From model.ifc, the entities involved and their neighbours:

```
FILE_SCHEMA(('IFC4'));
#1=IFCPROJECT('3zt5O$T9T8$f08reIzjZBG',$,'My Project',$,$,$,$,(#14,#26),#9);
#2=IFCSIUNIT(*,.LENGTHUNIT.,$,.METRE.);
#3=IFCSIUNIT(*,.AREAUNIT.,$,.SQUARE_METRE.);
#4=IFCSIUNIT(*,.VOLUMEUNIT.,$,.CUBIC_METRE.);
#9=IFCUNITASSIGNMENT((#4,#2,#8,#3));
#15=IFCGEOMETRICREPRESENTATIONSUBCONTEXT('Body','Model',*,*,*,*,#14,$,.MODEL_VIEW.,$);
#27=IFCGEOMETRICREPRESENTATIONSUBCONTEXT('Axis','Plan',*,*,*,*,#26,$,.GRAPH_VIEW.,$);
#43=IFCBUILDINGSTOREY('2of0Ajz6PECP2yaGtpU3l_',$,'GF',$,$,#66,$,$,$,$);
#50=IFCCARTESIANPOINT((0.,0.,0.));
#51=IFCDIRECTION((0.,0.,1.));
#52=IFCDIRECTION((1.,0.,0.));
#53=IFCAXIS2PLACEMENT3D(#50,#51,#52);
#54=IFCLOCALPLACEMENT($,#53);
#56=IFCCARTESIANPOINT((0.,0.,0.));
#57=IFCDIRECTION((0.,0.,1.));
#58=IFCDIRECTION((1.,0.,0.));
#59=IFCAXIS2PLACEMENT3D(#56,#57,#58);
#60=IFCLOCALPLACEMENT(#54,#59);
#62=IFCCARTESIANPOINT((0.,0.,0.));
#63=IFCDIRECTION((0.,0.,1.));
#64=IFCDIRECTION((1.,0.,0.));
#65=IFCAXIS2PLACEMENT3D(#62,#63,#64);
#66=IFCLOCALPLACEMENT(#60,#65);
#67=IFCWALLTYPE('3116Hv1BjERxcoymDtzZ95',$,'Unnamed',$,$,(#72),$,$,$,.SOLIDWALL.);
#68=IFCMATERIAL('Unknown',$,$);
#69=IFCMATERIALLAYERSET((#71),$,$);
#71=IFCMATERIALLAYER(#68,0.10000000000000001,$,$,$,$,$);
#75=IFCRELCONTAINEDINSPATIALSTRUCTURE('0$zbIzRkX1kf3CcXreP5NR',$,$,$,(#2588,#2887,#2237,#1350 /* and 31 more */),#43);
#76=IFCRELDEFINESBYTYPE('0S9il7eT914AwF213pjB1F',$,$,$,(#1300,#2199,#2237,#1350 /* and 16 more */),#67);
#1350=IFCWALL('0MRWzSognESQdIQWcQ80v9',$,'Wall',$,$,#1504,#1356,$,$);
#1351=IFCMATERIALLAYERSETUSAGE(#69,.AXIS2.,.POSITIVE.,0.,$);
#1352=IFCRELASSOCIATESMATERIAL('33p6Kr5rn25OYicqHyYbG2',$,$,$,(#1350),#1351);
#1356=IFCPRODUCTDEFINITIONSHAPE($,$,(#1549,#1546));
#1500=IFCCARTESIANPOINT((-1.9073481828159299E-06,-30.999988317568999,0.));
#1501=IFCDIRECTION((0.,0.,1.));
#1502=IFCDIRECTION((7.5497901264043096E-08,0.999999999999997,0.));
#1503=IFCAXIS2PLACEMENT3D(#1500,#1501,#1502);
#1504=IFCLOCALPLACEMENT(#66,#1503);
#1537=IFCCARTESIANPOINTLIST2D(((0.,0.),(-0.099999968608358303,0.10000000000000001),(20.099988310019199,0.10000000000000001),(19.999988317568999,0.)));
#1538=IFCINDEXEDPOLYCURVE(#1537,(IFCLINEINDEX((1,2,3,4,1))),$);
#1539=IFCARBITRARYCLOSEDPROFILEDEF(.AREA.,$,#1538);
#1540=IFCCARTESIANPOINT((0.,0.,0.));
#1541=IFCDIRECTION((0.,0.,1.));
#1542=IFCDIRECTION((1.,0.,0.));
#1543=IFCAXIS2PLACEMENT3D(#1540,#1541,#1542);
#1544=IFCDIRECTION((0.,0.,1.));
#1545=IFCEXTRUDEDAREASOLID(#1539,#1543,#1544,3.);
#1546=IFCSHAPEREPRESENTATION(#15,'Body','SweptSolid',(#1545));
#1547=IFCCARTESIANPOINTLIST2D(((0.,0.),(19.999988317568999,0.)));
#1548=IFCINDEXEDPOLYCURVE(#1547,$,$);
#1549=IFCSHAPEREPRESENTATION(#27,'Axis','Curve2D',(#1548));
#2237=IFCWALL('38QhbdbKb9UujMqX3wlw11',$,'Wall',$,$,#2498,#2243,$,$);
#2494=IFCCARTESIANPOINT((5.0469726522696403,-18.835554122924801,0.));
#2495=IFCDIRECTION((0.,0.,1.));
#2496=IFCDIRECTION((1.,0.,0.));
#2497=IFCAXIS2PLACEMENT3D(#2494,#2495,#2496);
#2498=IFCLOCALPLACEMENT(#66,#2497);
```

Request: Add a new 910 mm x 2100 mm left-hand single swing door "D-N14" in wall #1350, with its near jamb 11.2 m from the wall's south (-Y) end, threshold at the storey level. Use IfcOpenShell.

```python
import numpy as np
import ifcopenshell
import ifcopenshell.api.feature
import ifcopenshell.api.geometry
import ifcopenshell.api.root
import ifcopenshell.api.spatial
import ifcopenshell.geom
import ifcopenshell.util.element
import ifcopenshell.util.placement
import ifcopenshell.util.representation
import ifcopenshell.util.shape
import ifcopenshell.util.unit

model = ifcopenshell.open("model.ifc")
unit_scale = ifcopenshell.util.unit.calculate_unit_scale(model)
settings = ifcopenshell.geom.settings()


def volume(element):
    """Net volume in cubic metres, openings subtracted."""
    shape = ifcopenshell.geom.create_shape(settings, element)
    return ifcopenshell.util.shape.get_volume(shape.geometry)


wall = model.by_guid("0MRWzSognESQdIQWcQ80v9")
storey = ifcopenshell.util.element.get_container(wall, ifc_class="IfcBuildingStorey")
context = ifcopenshell.util.representation.get_context(model, "Model", "Body", "MODEL_VIEW")
before = volume(wall)

width, height, from_end, sill = 0.91, 2.1, 11.2, 0.0  # metres

# The wall runs along its own X axis, and the end named is its -X end.
wall_shape = ifcopenshell.geom.create_shape(settings, wall)
x, y, z = ifcopenshell.util.shape.get_vertices(wall_shape.geometry).T
start = x.min() + from_end
face, thickness = float(y.min()), float(y.max() - y.min())
wall_matrix = ifcopenshell.util.placement.get_local_placement(wall.ObjectPlacement)
level = ifcopenshell.util.placement.get_local_placement(storey.ObjectPlacement)[2, 3]


def in_wall(x, y):
    """Placement at x, y metres in the wall's axes, at sill height."""
    matrix = wall_matrix.copy()
    matrix[:, 3] = wall_matrix @ np.array([x / unit_scale, y / unit_scale, 0.0, 1.0])
    matrix[2, 3] = level + sill / unit_scale
    return matrix


# Opening: a box that overshoots both wall faces by 50 mm.
opening = ifcopenshell.api.root.create_entity(model, ifc_class="IfcOpeningElement", predefined_type="OPENING")
box = ifcopenshell.api.geometry.add_wall_representation(
    model, context=context, length=width, height=height, thickness=thickness + 0.1
)
ifcopenshell.api.geometry.assign_representation(model, product=opening, representation=box)
ifcopenshell.api.geometry.edit_object_placement(model, product=opening, matrix=in_wall(start, face - 0.05), is_si=False)
ifcopenshell.api.feature.add_feature(model, feature=opening, element=wall)

door = ifcopenshell.api.root.create_entity(model, ifc_class="IfcDoor", name="D-N14", predefined_type="DOOR")
door.OverallWidth, door.OverallHeight = width / unit_scale, height / unit_scale
door.OperationType = "SINGLE_SWING_LEFT"
body = ifcopenshell.api.geometry.add_door_representation(
    model,
    context=context,
    overall_width=door.OverallWidth,
    overall_height=door.OverallHeight,
    operation_type="SINGLE_SWING_LEFT",
    lining_properties={"LiningDepth": thickness / unit_scale, "ThresholdDepth": thickness / unit_scale},
)
ifcopenshell.api.geometry.assign_representation(model, product=door, representation=body)
ifcopenshell.api.spatial.assign_container(model, products=[door], relating_structure=storey)
ifcopenshell.api.feature.add_filling(model, opening=opening, element=door)

# The lining spans the wall, so the door starts at the wall face.
ifcopenshell.api.geometry.edit_object_placement(model, product=door, matrix=in_wall(start, face), is_si=False)

after = volume(wall)

print(f"wall volume {before:.3f} -> {after:.3f} m3")

model.write("model-out.ifc")
```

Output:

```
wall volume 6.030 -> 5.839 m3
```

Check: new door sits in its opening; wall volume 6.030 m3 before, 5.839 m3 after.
